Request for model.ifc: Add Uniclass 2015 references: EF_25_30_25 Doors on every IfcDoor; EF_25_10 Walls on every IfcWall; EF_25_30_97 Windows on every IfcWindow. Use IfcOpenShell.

First a look at what the model holds.

```python
import ifcopenshell

model = ifcopenshell.open("model.ifc")
print(model.schema)
print("classifications:", [c.Name for c in model.by_type("IfcClassification")])
for ifc_class in ("IfcDoor", "IfcRoof", "IfcStair", "IfcWall", "IfcWindow"):
    print(ifc_class, len(model.by_type(ifc_class)))
```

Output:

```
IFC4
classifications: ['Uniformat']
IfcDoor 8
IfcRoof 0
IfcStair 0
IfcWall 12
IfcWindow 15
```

```python
import ifcopenshell
import ifcopenshell.api.classification

model = ifcopenshell.open("model.ifc")

system = ifcopenshell.api.classification.add_classification(model, classification="Uniclass 2015")

codes = {
    "IfcDoor": ("EF_25_30_25", "Doors"),
    "IfcWall": ("EF_25_10", "Walls"),
    "IfcWindow": ("EF_25_30_97", "Windows"),
}
for ifc_class, (code, name) in codes.items():
    products = model.by_type(ifc_class)
    ifcopenshell.api.classification.add_reference(
        model, products=products, classification=system, identification=code, name=name
    )
    print(code, len(products))

model.write("model_v2.ifc")
```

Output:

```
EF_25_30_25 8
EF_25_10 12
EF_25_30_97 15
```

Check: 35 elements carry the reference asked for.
